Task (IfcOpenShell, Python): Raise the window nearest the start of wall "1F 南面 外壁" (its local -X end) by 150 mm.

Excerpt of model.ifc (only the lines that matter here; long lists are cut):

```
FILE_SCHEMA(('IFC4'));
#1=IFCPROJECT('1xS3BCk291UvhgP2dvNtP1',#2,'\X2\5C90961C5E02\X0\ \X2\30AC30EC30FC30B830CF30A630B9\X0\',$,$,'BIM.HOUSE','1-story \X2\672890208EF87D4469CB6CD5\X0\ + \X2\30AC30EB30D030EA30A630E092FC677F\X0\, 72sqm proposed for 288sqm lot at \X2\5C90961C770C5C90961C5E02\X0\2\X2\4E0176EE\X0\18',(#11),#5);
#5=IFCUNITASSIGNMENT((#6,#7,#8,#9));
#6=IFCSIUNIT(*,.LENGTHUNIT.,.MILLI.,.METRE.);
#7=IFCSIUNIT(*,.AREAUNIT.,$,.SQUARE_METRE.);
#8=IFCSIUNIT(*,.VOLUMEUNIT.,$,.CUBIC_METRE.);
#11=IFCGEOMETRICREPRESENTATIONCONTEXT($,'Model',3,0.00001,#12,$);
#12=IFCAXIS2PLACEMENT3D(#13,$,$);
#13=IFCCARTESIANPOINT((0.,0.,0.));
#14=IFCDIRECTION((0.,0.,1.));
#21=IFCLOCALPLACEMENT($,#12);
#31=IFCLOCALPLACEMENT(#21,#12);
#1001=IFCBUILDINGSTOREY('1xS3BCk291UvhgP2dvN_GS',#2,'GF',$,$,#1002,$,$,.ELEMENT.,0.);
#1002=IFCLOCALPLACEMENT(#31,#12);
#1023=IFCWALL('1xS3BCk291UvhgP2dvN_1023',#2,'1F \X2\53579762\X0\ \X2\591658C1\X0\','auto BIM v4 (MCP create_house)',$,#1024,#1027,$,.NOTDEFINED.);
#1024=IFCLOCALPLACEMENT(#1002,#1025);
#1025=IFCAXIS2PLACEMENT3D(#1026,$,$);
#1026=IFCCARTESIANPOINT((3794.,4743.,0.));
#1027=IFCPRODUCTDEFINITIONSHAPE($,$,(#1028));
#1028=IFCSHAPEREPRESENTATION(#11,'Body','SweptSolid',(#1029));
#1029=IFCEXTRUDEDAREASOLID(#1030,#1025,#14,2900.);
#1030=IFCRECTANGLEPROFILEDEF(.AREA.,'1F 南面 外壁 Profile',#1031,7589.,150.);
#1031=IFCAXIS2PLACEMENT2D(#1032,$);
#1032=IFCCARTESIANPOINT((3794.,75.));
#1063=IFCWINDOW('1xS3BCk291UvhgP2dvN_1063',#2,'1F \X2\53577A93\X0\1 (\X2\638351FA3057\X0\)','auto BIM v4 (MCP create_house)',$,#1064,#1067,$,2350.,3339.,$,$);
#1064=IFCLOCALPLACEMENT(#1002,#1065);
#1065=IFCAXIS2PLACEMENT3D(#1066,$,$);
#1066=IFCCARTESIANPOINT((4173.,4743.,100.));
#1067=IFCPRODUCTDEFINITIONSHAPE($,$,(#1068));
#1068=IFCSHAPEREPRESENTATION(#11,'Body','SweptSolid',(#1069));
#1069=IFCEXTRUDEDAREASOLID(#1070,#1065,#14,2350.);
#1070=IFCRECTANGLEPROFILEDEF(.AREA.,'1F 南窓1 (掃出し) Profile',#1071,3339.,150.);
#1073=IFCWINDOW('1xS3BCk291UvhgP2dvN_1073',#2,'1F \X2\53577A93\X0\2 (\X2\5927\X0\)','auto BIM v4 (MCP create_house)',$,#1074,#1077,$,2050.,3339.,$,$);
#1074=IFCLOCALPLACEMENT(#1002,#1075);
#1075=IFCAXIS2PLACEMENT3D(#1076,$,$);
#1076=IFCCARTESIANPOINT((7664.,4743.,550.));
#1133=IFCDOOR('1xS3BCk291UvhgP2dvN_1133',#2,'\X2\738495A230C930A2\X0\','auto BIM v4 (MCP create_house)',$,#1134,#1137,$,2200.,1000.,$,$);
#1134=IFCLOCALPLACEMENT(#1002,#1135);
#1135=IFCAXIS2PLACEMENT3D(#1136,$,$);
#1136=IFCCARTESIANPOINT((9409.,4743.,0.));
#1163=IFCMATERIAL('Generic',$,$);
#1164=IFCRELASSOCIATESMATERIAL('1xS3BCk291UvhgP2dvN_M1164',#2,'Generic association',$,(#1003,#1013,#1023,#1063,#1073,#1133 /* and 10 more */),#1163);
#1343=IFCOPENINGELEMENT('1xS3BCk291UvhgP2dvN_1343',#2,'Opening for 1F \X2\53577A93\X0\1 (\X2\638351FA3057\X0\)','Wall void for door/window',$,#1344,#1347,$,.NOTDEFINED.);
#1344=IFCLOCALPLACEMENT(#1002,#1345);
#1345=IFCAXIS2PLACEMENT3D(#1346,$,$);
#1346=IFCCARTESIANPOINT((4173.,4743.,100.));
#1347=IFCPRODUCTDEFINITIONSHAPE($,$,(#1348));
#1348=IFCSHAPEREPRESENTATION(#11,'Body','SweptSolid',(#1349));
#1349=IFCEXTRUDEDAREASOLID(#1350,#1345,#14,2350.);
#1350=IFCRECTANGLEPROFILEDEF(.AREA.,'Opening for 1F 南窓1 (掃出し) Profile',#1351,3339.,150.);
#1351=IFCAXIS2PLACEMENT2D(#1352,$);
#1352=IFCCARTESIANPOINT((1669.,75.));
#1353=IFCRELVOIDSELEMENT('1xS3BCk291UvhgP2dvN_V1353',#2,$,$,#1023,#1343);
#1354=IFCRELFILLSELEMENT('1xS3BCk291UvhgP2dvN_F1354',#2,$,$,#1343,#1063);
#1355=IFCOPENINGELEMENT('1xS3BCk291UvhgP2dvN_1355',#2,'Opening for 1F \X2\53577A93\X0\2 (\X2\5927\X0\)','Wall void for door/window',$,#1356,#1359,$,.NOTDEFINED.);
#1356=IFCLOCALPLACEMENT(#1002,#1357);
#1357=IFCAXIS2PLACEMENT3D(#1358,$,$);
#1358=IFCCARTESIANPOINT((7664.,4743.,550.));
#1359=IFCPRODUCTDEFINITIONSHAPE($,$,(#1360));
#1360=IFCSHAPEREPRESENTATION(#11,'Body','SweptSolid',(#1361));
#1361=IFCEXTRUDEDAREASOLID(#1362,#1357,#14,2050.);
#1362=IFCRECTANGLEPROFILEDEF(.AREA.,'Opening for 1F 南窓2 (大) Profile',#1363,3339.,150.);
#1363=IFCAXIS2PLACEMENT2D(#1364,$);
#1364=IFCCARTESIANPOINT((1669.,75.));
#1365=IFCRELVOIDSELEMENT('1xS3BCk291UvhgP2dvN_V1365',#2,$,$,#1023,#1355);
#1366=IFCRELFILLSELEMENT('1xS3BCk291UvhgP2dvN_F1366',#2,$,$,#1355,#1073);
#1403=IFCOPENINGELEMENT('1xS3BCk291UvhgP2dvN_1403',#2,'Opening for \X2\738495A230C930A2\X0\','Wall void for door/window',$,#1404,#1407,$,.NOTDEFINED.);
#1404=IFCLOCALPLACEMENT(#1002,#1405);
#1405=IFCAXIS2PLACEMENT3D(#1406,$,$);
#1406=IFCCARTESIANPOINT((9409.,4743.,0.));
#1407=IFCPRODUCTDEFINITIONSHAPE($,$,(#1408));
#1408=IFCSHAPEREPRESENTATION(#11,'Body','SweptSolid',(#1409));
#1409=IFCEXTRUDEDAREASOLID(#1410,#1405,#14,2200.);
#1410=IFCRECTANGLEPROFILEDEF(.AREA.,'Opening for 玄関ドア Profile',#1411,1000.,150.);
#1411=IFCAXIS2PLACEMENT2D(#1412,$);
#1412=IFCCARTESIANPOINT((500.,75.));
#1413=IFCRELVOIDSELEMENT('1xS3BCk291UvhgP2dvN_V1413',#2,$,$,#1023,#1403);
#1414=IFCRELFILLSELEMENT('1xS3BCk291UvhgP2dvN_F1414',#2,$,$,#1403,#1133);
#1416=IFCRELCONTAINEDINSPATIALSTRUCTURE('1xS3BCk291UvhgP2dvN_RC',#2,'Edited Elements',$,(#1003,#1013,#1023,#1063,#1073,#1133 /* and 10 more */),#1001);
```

```python
import numpy as np
import ifcopenshell
import ifcopenshell.api.geometry
import ifcopenshell.util.placement
import ifcopenshell.util.unit

model = ifcopenshell.open("model.ifc")
unit_scale = ifcopenshell.util.unit.calculate_unit_scale(model)

window = model.by_guid("1xS3BCk291UvhgP2dvN_1063")
opening = window.FillsVoids[0].RelatingOpeningElement
dz = 150.0

shift = np.array([0.0, 0.0, dz])
# The window is not placed relative to its opening, so move both.
for product in (opening, window):
    matrix = ifcopenshell.util.placement.get_local_placement(product.ObjectPlacement)
    matrix[:3, 3] += shift
    ifcopenshell.api.geometry.edit_object_placement(model, product=product, matrix=matrix, is_si=False)

print(f"moved by {dz * unit_scale:+.3f} m")

model.write("model_v2.ifc")
```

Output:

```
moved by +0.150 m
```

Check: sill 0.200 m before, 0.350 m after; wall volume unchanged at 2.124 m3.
